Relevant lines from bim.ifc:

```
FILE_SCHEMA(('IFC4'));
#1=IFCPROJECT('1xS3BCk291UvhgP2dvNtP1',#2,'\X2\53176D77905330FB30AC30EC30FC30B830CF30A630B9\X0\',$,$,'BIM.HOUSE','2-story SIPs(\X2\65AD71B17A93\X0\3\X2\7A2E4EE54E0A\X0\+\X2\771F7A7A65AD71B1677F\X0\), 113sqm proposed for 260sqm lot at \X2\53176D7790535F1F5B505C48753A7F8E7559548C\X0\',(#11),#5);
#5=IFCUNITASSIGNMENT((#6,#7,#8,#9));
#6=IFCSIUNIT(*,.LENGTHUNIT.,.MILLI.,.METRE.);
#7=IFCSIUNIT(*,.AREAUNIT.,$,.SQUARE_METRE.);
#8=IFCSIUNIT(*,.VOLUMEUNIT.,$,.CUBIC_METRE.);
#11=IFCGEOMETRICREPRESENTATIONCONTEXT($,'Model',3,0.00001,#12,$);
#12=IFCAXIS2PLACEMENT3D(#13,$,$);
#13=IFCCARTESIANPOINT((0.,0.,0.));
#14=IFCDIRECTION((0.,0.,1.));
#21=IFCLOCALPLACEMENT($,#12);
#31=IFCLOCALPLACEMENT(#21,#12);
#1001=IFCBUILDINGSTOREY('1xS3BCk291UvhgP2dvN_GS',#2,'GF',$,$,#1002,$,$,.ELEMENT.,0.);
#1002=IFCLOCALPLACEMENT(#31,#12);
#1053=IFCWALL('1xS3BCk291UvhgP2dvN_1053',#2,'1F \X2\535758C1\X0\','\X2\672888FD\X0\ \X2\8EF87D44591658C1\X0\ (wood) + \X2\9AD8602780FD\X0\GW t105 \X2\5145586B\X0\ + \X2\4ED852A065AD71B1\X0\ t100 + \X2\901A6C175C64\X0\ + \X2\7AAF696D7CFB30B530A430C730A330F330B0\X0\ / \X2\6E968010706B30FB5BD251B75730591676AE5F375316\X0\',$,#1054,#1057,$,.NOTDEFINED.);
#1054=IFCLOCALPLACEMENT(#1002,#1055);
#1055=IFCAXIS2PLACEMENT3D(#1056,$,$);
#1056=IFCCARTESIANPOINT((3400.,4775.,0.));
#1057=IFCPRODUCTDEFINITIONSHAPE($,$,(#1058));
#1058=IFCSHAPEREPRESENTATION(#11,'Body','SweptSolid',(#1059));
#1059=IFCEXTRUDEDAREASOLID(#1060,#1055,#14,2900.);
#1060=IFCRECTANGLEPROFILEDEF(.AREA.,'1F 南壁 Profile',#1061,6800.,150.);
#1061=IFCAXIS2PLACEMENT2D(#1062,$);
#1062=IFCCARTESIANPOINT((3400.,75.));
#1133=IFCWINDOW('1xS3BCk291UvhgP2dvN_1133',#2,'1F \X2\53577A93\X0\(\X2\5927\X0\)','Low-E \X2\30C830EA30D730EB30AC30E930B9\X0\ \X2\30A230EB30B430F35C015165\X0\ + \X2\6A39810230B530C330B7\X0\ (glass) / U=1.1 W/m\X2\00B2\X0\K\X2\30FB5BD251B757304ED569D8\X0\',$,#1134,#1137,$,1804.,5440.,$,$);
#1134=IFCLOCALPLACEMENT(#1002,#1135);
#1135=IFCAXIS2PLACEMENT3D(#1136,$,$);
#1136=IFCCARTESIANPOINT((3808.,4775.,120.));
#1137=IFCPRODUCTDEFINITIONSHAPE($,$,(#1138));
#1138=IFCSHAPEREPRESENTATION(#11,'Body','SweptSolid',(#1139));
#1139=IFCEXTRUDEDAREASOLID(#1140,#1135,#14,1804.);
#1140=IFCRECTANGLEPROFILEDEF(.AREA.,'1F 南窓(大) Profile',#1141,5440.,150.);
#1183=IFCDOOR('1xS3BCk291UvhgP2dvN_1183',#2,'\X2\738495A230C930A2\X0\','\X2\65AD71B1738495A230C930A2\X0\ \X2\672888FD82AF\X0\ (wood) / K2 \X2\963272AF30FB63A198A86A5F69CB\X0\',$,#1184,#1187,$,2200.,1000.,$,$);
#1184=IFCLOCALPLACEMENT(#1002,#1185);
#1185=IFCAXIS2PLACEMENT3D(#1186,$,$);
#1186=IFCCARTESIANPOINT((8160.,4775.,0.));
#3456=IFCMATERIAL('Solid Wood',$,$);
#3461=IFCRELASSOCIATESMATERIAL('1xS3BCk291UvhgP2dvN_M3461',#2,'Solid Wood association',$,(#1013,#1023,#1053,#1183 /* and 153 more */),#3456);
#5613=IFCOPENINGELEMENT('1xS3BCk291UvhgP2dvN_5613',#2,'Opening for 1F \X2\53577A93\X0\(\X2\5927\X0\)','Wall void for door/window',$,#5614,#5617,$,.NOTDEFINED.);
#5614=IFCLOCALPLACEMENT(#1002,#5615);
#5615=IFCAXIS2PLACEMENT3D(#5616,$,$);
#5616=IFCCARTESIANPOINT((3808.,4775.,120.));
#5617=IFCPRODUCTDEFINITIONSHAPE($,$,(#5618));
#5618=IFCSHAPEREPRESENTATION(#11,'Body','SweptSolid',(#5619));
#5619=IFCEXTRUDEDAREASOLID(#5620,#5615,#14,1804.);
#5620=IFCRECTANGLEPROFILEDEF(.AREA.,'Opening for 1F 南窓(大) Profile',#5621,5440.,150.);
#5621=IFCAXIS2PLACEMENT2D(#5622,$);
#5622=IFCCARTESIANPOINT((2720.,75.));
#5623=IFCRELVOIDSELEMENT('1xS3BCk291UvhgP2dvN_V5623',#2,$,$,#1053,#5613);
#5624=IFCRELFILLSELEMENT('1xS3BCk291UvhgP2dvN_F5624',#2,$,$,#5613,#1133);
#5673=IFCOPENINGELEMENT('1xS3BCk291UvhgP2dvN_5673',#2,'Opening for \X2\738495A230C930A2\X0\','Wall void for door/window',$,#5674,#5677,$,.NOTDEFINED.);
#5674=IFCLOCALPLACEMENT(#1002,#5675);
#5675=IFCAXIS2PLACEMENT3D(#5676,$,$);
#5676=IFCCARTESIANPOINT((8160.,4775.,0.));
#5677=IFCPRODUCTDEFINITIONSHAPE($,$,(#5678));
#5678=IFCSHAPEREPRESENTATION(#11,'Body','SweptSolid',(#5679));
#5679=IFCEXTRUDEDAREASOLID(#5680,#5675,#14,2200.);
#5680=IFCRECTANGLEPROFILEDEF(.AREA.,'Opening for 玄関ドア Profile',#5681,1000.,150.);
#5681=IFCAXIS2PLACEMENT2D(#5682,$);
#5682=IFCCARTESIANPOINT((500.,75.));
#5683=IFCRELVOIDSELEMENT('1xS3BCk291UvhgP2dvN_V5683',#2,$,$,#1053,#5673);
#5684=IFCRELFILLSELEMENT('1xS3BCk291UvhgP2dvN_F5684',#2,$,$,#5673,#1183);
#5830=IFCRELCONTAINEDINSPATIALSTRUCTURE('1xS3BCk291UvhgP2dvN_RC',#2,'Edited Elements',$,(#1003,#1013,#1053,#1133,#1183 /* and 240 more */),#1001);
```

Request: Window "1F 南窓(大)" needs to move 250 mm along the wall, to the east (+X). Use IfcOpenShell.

```python
import ifcopenshell
import ifcopenshell.api.geometry
import ifcopenshell.util.placement
import ifcopenshell.util.unit

model = ifcopenshell.open("bim.ifc")
unit_scale = ifcopenshell.util.unit.calculate_unit_scale(model)

window = model.by_guid("1xS3BCk291UvhgP2dvN_1133")
opening = window.FillsVoids[0].RelatingOpeningElement
wall = opening.VoidsElements[0].RelatingBuildingElement

wall_matrix = ifcopenshell.util.placement.get_local_placement(wall.ObjectPlacement)
shift = wall_matrix[:3, 0] * 0.25 / unit_scale
before = ifcopenshell.util.placement.get_local_placement(window.ObjectPlacement)[:3, 3].copy()

# The window is not placed relative to its opening, so move both.
for product in (opening, window):
    matrix = ifcopenshell.util.placement.get_local_placement(product.ObjectPlacement)
    matrix[:3, 3] += shift
    ifcopenshell.api.geometry.edit_object_placement(model, product=product, matrix=matrix, is_si=False)

after = ifcopenshell.util.placement.get_local_placement(window.ObjectPlacement)[:3, 3]
print("window moved by", (after - before).round(3) + 0.0)

model.write("bim_v2.ifc")
```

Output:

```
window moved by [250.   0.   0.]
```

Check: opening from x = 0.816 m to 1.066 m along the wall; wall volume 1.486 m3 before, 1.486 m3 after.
